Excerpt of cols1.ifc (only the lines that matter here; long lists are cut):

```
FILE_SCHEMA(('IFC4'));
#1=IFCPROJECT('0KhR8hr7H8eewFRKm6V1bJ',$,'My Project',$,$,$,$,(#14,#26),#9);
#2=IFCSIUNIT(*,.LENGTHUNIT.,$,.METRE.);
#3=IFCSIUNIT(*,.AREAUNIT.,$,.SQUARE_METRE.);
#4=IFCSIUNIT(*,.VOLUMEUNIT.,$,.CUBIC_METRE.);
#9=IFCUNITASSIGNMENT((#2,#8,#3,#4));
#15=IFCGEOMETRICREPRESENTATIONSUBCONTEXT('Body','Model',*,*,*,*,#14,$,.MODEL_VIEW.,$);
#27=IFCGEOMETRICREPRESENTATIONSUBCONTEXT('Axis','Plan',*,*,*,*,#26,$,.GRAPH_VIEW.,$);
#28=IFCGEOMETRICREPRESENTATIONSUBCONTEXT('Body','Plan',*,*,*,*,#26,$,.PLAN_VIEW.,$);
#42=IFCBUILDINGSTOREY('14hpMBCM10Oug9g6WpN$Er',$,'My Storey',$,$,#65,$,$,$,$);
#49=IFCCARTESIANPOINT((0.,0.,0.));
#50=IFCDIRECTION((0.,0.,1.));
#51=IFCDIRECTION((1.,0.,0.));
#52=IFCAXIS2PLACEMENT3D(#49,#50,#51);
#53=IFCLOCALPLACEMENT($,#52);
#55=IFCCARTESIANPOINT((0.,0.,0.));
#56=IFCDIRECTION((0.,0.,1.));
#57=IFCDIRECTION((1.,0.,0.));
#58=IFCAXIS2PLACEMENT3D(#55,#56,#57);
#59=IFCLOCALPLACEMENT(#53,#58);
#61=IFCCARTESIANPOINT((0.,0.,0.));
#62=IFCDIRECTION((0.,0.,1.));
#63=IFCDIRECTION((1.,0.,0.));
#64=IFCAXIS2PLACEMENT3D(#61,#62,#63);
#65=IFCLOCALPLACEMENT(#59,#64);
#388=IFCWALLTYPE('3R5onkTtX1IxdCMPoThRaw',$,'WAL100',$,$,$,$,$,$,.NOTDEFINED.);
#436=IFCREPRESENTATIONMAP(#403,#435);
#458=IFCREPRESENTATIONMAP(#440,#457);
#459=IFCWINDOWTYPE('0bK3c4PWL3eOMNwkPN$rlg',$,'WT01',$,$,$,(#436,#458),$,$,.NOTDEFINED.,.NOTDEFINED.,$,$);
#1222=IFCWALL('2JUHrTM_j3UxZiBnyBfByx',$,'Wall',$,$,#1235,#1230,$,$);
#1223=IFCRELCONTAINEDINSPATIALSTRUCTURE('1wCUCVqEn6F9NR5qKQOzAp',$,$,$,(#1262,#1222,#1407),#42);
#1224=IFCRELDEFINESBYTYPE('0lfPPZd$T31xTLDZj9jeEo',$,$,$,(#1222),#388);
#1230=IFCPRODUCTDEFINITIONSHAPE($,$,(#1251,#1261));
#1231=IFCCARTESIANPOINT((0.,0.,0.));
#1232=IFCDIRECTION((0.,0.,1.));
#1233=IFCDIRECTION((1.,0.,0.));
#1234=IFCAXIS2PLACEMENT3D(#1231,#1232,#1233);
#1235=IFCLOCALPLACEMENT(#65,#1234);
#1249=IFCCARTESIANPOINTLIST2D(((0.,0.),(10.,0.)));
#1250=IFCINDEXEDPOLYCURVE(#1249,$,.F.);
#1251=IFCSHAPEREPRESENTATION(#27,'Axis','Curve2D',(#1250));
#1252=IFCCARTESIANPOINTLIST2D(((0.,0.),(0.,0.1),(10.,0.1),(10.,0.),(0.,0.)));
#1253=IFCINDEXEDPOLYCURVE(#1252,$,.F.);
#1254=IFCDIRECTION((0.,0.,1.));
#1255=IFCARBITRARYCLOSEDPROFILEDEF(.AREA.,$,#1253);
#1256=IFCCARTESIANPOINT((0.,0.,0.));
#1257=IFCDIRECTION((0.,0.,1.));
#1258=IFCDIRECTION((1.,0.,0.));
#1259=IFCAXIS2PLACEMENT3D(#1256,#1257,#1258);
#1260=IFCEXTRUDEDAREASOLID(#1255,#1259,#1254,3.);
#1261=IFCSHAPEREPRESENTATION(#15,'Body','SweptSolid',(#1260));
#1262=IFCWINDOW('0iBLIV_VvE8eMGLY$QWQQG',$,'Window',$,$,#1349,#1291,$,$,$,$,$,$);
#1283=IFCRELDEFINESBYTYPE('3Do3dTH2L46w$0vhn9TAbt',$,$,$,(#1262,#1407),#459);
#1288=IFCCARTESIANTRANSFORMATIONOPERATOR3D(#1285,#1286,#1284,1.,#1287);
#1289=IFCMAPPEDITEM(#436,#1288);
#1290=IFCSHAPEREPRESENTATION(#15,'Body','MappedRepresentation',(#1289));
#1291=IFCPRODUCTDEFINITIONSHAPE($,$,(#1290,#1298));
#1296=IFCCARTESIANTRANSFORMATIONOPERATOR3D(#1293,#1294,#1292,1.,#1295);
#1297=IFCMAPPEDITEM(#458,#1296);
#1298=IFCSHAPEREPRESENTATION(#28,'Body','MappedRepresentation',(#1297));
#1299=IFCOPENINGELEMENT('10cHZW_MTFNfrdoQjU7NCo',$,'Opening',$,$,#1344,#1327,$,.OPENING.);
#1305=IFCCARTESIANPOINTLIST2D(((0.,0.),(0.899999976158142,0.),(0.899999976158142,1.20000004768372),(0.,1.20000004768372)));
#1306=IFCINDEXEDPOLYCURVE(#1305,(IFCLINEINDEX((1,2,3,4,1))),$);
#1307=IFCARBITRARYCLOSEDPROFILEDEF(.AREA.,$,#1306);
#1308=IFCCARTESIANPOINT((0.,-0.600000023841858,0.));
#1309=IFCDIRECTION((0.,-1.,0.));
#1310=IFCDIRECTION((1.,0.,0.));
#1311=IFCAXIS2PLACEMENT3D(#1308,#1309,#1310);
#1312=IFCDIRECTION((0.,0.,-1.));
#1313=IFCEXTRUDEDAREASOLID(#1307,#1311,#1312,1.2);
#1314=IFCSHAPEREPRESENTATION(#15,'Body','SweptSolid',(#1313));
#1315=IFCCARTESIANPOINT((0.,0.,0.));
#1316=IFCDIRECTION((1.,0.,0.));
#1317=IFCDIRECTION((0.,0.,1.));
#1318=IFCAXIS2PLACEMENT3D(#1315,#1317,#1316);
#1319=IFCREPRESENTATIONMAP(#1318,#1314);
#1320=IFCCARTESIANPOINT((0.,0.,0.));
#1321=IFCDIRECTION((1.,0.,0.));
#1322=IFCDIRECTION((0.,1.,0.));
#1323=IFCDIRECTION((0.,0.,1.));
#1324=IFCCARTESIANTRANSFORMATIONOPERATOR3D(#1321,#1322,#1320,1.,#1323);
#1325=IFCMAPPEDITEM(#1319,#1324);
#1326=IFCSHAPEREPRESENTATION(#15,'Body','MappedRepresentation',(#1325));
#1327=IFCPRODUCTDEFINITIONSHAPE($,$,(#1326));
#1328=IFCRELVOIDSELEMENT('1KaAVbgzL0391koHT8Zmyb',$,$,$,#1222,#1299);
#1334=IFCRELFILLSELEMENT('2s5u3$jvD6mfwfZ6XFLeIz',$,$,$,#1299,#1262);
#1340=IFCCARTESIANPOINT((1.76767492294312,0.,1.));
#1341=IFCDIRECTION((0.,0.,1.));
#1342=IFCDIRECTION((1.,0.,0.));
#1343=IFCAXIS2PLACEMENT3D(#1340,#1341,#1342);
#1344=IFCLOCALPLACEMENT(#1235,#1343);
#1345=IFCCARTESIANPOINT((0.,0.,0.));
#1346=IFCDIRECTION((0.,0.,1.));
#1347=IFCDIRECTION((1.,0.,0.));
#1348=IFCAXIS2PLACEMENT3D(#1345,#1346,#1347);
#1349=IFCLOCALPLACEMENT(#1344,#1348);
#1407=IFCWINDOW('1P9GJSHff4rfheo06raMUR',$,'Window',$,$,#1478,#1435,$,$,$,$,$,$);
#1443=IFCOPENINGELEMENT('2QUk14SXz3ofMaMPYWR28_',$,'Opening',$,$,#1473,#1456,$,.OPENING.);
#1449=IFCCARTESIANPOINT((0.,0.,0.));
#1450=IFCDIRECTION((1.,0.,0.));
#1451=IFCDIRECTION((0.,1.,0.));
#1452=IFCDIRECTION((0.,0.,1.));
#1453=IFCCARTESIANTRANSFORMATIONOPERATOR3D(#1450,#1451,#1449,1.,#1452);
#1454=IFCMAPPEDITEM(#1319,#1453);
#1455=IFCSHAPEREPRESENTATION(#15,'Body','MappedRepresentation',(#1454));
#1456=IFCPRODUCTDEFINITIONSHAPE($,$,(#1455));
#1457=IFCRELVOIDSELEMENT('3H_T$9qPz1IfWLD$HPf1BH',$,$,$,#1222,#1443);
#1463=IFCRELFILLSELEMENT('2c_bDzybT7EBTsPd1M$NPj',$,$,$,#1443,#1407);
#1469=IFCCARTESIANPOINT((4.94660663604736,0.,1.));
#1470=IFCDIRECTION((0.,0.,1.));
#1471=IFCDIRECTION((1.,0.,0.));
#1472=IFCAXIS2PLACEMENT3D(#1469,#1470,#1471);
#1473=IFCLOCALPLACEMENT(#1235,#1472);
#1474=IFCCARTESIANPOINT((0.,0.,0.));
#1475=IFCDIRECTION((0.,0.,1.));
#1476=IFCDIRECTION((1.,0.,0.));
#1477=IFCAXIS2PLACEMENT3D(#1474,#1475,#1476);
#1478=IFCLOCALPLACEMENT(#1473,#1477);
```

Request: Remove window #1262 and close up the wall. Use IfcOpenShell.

```python
import ifcopenshell
import ifcopenshell.api.feature
import ifcopenshell.api.root
import ifcopenshell.geom
import ifcopenshell.util.shape

model = ifcopenshell.open("cols1.ifc")
settings = ifcopenshell.geom.settings()


def volume(element):
    """Net volume in cubic metres, openings subtracted."""
    shape = ifcopenshell.geom.create_shape(settings, element)
    return ifcopenshell.util.shape.get_volume(shape.geometry)


window = model.by_guid("0iBLIV_VvE8eMGLY$QWQQG")
opening = window.FillsVoids[0].RelatingOpeningElement
wall = opening.VoidsElements[0].RelatingBuildingElement
before = volume(wall)

ifcopenshell.api.root.remove_product(model, product=window)
ifcopenshell.api.feature.remove_feature(model, feature=opening)

after = volume(wall)

print(f"wall volume {before:.3f} -> {after:.3f} m3")

model.write("cols1_rev.ifc")
```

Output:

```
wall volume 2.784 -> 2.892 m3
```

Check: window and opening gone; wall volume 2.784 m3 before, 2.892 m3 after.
